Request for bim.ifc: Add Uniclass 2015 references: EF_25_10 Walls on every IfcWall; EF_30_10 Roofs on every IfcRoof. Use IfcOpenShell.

First a look at what the model holds.

```python
import ifcopenshell

model = ifcopenshell.open("bim.ifc")
print(model.schema)
print("classifications:", [c.Name for c in model.by_type("IfcClassification")])
for ifc_class in ("IfcDoor", "IfcRoof", "IfcStair", "IfcWall", "IfcWindow"):
    print(ifc_class, len(model.by_type(ifc_class)))
```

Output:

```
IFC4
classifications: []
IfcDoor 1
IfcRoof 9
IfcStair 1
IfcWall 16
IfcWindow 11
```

```python
import ifcopenshell
import ifcopenshell.api.classification

model = ifcopenshell.open("bim.ifc")

system = ifcopenshell.api.classification.add_classification(model, classification="Uniclass 2015")

codes = {
    "IfcWall": ("EF_25_10", "Walls"),
    "IfcRoof": ("EF_30_10", "Roofs"),
}
for ifc_class, (code, name) in codes.items():
    products = model.by_type(ifc_class)
    ifcopenshell.api.classification.add_reference(
        model, products=products, classification=system, identification=code, name=name
    )
    print(code, len(products))

model.write("bim_rev.ifc")
```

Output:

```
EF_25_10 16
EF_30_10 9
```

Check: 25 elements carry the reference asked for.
